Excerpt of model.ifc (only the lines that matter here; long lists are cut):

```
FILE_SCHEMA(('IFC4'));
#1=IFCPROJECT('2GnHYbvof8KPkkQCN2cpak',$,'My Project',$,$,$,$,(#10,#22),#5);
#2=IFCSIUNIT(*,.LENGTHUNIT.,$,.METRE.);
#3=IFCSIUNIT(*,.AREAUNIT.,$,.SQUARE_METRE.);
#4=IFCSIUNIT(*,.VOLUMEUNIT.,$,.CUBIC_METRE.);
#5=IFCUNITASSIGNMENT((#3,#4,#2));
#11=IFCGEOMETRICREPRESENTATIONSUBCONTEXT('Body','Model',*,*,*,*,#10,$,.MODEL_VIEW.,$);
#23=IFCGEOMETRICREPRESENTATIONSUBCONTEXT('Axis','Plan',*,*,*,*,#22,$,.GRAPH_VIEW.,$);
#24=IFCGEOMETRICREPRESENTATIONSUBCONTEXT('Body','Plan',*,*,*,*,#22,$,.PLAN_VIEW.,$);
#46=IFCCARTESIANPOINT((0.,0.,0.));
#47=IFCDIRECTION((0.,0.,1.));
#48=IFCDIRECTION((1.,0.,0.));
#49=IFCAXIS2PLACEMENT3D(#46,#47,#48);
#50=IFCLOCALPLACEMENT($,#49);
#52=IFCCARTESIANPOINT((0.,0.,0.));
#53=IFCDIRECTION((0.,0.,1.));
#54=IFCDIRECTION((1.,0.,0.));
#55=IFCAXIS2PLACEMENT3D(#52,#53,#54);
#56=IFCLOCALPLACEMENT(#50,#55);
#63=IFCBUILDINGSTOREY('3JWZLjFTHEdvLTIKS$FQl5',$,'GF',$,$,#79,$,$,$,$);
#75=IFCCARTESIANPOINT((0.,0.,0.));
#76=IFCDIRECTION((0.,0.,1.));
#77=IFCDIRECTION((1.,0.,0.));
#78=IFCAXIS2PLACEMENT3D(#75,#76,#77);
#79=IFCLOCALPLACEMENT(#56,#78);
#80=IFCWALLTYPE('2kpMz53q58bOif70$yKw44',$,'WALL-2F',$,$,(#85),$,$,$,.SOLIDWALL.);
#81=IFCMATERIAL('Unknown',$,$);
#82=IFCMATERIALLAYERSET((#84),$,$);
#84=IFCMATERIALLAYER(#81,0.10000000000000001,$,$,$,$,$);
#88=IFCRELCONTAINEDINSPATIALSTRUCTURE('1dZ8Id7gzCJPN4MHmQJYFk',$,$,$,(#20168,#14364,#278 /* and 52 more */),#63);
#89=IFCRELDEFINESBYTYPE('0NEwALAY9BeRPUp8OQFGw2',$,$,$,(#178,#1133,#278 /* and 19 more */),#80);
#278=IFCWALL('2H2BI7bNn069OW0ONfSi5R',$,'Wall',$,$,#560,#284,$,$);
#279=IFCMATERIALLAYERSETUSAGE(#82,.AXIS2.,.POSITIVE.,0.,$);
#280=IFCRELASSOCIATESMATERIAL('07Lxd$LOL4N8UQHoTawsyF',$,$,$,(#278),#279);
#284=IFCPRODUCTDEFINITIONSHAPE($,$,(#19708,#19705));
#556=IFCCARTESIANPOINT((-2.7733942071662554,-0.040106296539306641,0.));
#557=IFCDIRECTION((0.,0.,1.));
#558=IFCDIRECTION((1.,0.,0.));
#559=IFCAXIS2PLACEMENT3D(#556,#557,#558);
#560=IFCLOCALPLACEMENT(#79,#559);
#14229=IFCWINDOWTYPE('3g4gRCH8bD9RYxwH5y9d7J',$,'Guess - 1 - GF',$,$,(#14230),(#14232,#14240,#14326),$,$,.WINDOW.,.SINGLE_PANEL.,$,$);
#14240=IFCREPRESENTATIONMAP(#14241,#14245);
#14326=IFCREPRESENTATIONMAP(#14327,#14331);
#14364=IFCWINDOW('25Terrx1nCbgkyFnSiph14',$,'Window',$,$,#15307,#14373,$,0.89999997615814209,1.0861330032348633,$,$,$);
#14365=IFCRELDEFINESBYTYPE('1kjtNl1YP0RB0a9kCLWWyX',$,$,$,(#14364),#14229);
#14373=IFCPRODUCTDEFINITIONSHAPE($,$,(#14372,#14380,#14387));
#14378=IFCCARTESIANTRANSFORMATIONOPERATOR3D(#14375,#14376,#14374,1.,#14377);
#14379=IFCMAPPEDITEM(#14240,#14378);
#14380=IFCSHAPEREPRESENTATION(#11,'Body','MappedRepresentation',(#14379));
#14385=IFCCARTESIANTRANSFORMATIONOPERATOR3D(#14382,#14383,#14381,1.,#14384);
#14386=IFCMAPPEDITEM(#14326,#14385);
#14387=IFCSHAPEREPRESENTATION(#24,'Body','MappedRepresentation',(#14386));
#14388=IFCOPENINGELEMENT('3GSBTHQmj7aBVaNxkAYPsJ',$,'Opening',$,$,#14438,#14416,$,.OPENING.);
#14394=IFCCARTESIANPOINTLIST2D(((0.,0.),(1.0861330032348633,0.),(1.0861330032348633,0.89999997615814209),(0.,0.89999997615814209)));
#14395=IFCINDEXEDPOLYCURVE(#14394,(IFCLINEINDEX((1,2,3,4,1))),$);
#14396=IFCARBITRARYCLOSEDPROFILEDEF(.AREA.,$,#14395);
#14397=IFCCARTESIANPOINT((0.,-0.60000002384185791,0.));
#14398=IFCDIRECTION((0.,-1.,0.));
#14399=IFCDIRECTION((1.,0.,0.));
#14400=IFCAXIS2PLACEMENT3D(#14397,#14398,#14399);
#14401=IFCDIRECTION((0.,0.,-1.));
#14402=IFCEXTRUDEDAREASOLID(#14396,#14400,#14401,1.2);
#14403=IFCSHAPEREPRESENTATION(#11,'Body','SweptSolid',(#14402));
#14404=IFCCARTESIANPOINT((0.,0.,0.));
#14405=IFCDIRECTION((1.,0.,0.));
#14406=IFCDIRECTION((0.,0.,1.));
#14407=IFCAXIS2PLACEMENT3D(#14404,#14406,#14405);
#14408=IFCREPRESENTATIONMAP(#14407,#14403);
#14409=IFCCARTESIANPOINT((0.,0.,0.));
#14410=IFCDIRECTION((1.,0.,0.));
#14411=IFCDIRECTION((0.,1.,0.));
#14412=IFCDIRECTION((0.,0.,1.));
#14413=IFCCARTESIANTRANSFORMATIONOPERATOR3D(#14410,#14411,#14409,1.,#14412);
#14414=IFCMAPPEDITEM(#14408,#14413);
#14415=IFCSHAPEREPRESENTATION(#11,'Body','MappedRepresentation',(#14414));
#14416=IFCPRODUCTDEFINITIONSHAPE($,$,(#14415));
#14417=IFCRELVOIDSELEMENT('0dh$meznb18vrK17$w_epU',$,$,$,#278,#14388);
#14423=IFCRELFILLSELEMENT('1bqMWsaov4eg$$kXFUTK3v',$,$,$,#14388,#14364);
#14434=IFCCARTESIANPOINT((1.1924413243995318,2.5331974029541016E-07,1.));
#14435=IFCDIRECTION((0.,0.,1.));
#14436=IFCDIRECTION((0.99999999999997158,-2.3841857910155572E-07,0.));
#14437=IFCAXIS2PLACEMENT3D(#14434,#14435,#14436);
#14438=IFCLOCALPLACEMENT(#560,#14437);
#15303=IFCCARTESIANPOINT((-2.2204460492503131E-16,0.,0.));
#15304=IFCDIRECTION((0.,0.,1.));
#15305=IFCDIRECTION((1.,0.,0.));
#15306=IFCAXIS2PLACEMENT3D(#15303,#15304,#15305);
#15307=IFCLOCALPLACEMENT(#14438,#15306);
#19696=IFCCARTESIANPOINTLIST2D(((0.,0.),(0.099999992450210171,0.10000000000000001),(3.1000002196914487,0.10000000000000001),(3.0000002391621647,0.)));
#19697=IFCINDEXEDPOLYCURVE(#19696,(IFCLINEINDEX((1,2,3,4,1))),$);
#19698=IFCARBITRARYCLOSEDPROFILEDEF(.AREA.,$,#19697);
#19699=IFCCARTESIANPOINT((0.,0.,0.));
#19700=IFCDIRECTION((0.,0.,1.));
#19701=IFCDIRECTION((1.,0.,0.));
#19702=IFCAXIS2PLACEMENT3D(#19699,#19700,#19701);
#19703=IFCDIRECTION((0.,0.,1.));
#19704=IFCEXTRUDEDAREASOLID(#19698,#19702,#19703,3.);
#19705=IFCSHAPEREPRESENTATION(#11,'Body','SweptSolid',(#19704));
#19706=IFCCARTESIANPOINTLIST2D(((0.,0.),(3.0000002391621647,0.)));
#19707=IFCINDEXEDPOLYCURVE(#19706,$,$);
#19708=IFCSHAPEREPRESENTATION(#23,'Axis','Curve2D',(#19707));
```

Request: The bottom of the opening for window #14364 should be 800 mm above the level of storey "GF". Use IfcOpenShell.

```python
import numpy as np
import ifcopenshell
import ifcopenshell.api.geometry
import ifcopenshell.geom
import ifcopenshell.util.element
import ifcopenshell.util.placement
import ifcopenshell.util.shape
import ifcopenshell.util.unit

model = ifcopenshell.open("model.ifc")
unit_scale = ifcopenshell.util.unit.calculate_unit_scale(model)

window = model.by_guid("25Terrx1nCbgkyFnSiph14")
opening = window.FillsVoids[0].RelatingOpeningElement
storey = ifcopenshell.util.element.get_container(window, ifc_class="IfcBuildingStorey")
level = ifcopenshell.util.placement.get_local_placement(storey.ObjectPlacement)[2, 3]

# The opening's origin need not be at the sill, so measure its lowest point.
shape = ifcopenshell.geom.create_shape(ifcopenshell.geom.settings(), opening)
bottom = ifcopenshell.util.shape.get_shape_bottom_elevation(shape, shape.geometry) / unit_scale
dz = level + 0.8 / unit_scale - bottom

shift = np.array([0.0, 0.0, dz])
# The window is placed relative to its opening, so it follows when the opening moves.
matrix = ifcopenshell.util.placement.get_local_placement(opening.ObjectPlacement)
matrix[:3, 3] += shift
ifcopenshell.api.geometry.edit_object_placement(
    model, product=opening, matrix=matrix, is_si=False, should_transform_children=True
)

print(f"moved by {dz * unit_scale:+.3f} m")

model.write("model_updated.ifc")
```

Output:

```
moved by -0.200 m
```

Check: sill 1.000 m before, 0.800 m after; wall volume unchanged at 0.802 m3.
